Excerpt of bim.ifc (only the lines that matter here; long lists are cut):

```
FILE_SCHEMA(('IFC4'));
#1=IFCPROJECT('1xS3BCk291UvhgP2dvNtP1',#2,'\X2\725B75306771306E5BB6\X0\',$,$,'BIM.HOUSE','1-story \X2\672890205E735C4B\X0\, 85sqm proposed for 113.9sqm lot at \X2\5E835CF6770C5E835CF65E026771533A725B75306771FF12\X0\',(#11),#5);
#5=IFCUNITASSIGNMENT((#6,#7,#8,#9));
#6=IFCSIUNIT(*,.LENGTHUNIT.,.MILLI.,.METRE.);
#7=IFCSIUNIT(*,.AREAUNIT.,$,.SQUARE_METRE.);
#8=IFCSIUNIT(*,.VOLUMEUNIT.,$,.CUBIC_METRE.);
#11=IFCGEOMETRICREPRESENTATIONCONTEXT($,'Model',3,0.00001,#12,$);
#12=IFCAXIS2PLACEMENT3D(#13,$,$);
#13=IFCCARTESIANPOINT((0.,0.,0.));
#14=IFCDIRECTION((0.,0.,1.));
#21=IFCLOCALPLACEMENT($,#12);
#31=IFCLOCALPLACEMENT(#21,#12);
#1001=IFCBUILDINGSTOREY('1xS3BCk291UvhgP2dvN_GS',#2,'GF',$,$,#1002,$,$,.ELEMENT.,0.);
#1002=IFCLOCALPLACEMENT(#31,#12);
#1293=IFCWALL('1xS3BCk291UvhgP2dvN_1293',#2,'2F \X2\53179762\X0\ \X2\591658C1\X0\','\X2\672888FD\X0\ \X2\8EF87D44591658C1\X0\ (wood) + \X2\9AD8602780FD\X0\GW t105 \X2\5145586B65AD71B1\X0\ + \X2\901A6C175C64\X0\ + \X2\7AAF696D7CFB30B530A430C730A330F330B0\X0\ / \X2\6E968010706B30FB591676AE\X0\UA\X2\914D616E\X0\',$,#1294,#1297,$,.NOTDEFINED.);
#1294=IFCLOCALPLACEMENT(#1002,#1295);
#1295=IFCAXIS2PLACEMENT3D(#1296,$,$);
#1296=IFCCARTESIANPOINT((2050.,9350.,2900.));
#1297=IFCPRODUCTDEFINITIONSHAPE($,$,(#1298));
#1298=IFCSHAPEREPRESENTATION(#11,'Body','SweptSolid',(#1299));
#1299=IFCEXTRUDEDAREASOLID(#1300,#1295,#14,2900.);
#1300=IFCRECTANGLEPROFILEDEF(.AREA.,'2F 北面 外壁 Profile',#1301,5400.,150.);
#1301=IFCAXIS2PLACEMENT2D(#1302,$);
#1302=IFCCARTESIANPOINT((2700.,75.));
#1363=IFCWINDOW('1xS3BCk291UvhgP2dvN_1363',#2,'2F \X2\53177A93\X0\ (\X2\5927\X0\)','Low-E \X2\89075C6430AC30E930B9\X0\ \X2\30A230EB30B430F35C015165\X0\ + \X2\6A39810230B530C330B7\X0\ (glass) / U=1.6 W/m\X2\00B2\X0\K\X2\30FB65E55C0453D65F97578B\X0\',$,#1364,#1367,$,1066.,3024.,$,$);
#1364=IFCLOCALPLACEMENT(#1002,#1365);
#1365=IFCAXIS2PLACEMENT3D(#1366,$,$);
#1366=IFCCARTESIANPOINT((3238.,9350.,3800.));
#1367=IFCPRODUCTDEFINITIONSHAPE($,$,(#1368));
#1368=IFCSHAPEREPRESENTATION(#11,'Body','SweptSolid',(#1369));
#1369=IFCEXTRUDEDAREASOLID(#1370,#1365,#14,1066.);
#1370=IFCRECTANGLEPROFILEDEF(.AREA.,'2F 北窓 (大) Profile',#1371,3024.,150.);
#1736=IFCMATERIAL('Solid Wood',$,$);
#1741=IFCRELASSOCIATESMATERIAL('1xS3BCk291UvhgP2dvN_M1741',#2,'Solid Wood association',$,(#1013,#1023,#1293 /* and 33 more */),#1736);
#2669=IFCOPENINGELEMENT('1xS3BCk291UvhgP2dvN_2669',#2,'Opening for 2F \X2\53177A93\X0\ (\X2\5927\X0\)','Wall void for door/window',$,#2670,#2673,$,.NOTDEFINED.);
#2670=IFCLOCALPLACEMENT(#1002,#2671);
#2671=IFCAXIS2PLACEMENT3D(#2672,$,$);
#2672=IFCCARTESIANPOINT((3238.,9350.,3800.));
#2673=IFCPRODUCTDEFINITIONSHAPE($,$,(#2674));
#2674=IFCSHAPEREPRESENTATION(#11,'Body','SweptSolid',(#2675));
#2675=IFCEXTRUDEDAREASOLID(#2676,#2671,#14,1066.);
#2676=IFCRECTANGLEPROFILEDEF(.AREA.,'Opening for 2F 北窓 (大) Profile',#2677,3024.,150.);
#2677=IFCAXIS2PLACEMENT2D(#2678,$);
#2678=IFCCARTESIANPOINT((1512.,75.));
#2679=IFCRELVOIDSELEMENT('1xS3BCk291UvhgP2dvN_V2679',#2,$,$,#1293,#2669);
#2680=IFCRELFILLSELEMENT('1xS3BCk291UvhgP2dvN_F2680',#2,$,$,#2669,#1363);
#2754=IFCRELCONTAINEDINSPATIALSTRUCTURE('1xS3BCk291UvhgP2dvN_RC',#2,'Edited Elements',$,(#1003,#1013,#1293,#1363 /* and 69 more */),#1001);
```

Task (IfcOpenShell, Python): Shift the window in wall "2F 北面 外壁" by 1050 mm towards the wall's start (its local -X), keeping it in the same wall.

```python
import ifcopenshell
import ifcopenshell.api.geometry
import ifcopenshell.util.placement
import ifcopenshell.util.unit

model = ifcopenshell.open("bim.ifc")
unit_scale = ifcopenshell.util.unit.calculate_unit_scale(model)

window = model.by_guid("1xS3BCk291UvhgP2dvN_1363")
opening = window.FillsVoids[0].RelatingOpeningElement
wall = opening.VoidsElements[0].RelatingBuildingElement

wall_matrix = ifcopenshell.util.placement.get_local_placement(wall.ObjectPlacement)
shift = wall_matrix[:3, 0] * -1.05 / unit_scale
before = ifcopenshell.util.placement.get_local_placement(window.ObjectPlacement)[:3, 3].copy()

# The window is not placed relative to its opening, so move both.
for product in (opening, window):
    matrix = ifcopenshell.util.placement.get_local_placement(product.ObjectPlacement)
    matrix[:3, 3] += shift
    ifcopenshell.api.geometry.edit_object_placement(model, product=product, matrix=matrix, is_si=False)

after = ifcopenshell.util.placement.get_local_placement(window.ObjectPlacement)[:3, 3]
print("window moved by", (after - before).round(3) + 0.0)

model.write("bim_updated.ifc")
```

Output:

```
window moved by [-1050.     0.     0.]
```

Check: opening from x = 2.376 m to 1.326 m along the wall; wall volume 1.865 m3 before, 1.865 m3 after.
